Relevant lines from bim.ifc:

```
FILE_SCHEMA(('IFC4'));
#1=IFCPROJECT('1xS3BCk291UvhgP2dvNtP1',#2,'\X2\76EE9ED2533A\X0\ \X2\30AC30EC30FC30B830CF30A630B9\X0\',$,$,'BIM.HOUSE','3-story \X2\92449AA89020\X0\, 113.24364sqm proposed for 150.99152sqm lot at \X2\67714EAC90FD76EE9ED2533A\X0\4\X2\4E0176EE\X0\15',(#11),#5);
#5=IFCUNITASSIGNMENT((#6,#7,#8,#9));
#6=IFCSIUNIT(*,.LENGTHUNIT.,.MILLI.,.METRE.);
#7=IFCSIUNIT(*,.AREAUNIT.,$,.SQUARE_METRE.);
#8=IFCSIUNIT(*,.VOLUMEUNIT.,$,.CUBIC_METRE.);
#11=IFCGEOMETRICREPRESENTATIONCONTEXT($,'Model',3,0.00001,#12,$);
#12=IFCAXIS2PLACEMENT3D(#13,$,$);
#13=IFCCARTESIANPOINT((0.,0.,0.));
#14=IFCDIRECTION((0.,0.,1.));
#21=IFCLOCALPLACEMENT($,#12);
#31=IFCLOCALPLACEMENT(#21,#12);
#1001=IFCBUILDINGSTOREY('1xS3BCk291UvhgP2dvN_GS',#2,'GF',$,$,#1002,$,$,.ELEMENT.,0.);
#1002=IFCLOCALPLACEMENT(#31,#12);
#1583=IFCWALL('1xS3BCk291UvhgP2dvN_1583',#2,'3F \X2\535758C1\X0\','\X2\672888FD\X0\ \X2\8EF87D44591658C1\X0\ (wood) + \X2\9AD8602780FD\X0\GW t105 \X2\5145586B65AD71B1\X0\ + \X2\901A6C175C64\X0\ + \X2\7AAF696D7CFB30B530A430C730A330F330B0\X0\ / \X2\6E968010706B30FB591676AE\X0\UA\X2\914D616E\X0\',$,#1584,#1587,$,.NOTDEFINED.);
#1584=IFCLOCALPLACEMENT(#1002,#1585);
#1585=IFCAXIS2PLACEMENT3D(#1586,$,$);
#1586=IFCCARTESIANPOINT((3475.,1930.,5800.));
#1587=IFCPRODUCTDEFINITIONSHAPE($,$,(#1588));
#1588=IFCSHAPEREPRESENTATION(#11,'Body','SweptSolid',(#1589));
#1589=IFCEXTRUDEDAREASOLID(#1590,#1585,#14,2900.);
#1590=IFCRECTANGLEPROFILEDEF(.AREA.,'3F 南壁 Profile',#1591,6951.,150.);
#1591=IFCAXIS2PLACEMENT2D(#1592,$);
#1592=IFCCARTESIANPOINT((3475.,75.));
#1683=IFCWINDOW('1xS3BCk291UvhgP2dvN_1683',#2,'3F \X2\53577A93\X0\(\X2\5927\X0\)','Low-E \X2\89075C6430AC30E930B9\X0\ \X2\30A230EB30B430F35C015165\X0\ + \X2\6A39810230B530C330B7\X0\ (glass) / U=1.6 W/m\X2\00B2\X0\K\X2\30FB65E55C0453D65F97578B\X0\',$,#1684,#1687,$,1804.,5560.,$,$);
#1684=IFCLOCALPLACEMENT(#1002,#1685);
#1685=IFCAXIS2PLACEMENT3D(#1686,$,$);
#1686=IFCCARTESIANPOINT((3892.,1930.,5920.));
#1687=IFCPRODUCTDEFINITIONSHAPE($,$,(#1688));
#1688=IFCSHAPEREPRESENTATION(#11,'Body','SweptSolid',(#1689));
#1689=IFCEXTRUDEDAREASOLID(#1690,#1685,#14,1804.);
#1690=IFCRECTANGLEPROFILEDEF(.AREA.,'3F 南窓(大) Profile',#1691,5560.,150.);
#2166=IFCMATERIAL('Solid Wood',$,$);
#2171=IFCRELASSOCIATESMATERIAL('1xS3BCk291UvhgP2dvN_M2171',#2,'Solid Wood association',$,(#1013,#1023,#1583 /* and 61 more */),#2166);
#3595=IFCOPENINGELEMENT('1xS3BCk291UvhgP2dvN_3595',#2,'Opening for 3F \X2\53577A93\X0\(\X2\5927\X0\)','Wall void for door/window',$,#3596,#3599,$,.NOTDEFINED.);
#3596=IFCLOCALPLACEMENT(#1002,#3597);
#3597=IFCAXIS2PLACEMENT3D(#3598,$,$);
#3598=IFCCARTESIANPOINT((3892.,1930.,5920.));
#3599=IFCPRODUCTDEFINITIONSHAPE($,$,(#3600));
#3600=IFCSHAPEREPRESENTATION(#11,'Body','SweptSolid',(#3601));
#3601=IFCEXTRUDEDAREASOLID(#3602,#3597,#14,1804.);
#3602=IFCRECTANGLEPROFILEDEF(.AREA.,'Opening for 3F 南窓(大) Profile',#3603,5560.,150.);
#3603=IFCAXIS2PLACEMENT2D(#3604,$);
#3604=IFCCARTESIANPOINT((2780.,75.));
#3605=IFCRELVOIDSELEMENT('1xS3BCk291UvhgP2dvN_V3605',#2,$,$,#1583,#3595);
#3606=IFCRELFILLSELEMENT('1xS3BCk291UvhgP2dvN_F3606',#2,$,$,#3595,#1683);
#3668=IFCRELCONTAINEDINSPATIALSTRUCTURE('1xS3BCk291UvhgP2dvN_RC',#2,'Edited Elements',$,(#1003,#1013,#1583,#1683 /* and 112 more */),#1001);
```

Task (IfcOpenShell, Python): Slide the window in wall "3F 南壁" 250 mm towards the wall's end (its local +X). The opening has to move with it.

```python
import ifcopenshell
import ifcopenshell.api.geometry
import ifcopenshell.util.placement
import ifcopenshell.util.unit

model = ifcopenshell.open("bim.ifc")
unit_scale = ifcopenshell.util.unit.calculate_unit_scale(model)

window = model.by_guid("1xS3BCk291UvhgP2dvN_1683")
opening = window.FillsVoids[0].RelatingOpeningElement
wall = opening.VoidsElements[0].RelatingBuildingElement

wall_matrix = ifcopenshell.util.placement.get_local_placement(wall.ObjectPlacement)
shift = wall_matrix[:3, 0] * 0.25 / unit_scale
before = ifcopenshell.util.placement.get_local_placement(window.ObjectPlacement)[:3, 3].copy()

# The window is not placed relative to its opening, so move both.
for product in (opening, window):
    matrix = ifcopenshell.util.placement.get_local_placement(product.ObjectPlacement)
    matrix[:3, 3] += shift
    ifcopenshell.api.geometry.edit_object_placement(model, product=product, matrix=matrix, is_si=False)

after = ifcopenshell.util.placement.get_local_placement(window.ObjectPlacement)[:3, 3]
print("window moved by", (after - before).round(3) + 0.0)

model.write("bim_edited.ifc")
```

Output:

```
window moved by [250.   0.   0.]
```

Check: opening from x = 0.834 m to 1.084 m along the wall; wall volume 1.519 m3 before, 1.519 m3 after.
